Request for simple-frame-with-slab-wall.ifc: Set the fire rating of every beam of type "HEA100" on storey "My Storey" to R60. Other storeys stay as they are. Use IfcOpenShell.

First a look at what the model holds.

```python
import ifcopenshell
import ifcopenshell.util.element

model = ifcopenshell.open("simple-frame-with-slab-wall.ifc")
print(model.schema)
storey = next(s for s in model.by_type("IfcBuildingStorey") if s.Name == "My Storey")
beams = [e for e in ifcopenshell.util.element.get_decomposition(storey) if e.is_a("IfcBeam")]
seen = {}
for e in beams:
    element_type = ifcopenshell.util.element.get_type(e)
    key = (element_type.Name if element_type != e and element_type else None, ifcopenshell.util.element.get_pset(e, "Pset_BeamCommon", "FireRating"))
    seen[key] = seen.get(key, 0) + 1
for (name, value), count in sorted(seen.items(), key=str):
    print(count, "x", name, "|", value)
```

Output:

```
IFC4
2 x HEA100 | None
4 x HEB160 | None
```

```python
import ifcopenshell
import ifcopenshell.api.pset
import ifcopenshell.util.element

model = ifcopenshell.open("simple-frame-with-slab-wall.ifc")

storey = next(s for s in model.by_type("IfcBuildingStorey") if s.Name == "My Storey")
beams = [e for e in ifcopenshell.util.element.get_decomposition(storey) if e.is_a("IfcBeam")]

count = 0
for e in beams:
    element_type = ifcopenshell.util.element.get_type(e)
    if element_type in (None, e) or element_type.Name != "HEA100":
        continue
    # add_pset returns the element's existing set when there is one.
    pset = ifcopenshell.api.pset.add_pset(model, product=e, name="Pset_BeamCommon")
    ifcopenshell.api.pset.edit_pset(model, pset=pset, properties={"FireRating": "R60"})
    count += 1

print(count, "beams updated")

model.write("simple-frame-with-slab-wall_updated.ifc")
```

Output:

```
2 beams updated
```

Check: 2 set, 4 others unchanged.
